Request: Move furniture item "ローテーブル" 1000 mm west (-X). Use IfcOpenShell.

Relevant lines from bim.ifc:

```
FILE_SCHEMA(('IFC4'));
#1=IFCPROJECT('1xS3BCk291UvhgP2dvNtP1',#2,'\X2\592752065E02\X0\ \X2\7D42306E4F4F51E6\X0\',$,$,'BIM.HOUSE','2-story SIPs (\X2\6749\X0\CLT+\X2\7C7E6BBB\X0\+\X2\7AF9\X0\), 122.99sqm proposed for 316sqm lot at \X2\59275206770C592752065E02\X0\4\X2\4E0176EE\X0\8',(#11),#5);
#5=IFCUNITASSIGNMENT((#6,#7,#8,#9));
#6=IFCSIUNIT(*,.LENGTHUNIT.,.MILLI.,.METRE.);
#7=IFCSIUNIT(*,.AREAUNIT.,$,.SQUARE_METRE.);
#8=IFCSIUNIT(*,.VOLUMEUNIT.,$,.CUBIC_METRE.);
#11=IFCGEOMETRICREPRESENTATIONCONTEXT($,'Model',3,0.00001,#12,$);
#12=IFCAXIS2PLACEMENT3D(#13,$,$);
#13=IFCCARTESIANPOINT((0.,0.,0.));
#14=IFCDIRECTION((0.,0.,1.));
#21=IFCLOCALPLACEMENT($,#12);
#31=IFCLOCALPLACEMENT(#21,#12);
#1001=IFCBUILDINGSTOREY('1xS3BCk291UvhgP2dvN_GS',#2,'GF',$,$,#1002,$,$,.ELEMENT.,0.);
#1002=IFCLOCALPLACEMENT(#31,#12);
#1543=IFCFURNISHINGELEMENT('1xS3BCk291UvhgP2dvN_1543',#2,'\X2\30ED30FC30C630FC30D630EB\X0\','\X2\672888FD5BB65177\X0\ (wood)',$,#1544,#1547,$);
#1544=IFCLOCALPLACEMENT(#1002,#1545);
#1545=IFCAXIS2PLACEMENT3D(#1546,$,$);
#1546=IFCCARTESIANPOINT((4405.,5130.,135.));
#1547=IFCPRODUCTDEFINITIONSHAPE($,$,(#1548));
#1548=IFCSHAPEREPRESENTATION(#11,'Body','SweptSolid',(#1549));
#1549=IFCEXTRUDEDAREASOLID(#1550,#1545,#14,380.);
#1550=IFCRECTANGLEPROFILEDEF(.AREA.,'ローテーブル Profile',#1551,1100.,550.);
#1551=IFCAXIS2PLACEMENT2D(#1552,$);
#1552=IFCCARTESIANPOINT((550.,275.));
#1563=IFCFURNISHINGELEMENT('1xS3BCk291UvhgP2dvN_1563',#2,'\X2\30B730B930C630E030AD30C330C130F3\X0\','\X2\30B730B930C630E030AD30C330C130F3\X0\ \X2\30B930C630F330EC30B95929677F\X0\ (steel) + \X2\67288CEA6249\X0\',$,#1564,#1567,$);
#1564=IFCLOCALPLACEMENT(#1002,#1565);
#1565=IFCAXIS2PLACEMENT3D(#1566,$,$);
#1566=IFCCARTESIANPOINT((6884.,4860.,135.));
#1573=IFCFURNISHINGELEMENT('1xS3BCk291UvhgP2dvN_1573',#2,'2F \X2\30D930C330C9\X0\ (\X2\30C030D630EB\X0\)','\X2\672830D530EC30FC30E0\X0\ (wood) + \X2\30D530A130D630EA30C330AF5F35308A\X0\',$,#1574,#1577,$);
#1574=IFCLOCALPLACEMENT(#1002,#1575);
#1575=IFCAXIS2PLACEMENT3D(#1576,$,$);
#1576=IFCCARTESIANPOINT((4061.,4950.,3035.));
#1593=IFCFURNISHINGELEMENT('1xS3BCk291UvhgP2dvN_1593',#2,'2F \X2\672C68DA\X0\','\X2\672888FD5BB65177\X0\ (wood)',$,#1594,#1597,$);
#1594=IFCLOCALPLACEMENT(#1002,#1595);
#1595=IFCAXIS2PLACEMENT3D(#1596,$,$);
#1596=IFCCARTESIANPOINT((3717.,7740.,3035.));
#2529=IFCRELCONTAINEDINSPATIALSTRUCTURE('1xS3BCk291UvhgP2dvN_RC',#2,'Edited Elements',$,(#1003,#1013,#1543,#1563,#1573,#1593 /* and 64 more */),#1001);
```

```python
import ifcopenshell
import ifcopenshell.api.geometry
import ifcopenshell.util.placement

model = ifcopenshell.open("bim.ifc")

item = model.by_guid("1xS3BCk291UvhgP2dvN_1543")
matrix = ifcopenshell.util.placement.get_local_placement(item.ObjectPlacement)
matrix[0, 3] -= 1000.0
ifcopenshell.api.geometry.edit_object_placement(model, product=item, matrix=matrix, is_si=False)

print(ifcopenshell.util.placement.get_local_placement(item.ObjectPlacement).round(3) + 0.0)

model.write("bim_rev.ifc")
```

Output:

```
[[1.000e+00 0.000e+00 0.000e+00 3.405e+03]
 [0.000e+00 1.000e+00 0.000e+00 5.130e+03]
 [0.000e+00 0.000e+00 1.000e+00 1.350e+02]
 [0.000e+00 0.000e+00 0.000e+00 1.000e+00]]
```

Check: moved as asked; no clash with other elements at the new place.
